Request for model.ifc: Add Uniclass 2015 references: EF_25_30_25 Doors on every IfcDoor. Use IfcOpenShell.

First a look at what the model holds.

```python
import ifcopenshell

model = ifcopenshell.open("model.ifc")
print(model.schema)
print("classifications:", [c.Name for c in model.by_type("IfcClassification")])
for ifc_class in ("IfcDoor", "IfcRoof", "IfcStair", "IfcWall", "IfcWindow"):
    print(ifc_class, len(model.by_type(ifc_class)))
```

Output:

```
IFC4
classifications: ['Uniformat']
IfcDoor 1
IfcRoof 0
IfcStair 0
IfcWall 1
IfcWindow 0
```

```python
import ifcopenshell
import ifcopenshell.api.classification

model = ifcopenshell.open("model.ifc")

system = ifcopenshell.api.classification.add_classification(model, classification="Uniclass 2015")

codes = {
    "IfcDoor": ("EF_25_30_25", "Doors"),
}
for ifc_class, (code, name) in codes.items():
    products = model.by_type(ifc_class)
    ifcopenshell.api.classification.add_reference(
        model, products=products, classification=system, identification=code, name=name
    )
    print(code, len(products))

model.write("model-out.ifc")
```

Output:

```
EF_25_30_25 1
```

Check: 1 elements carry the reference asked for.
